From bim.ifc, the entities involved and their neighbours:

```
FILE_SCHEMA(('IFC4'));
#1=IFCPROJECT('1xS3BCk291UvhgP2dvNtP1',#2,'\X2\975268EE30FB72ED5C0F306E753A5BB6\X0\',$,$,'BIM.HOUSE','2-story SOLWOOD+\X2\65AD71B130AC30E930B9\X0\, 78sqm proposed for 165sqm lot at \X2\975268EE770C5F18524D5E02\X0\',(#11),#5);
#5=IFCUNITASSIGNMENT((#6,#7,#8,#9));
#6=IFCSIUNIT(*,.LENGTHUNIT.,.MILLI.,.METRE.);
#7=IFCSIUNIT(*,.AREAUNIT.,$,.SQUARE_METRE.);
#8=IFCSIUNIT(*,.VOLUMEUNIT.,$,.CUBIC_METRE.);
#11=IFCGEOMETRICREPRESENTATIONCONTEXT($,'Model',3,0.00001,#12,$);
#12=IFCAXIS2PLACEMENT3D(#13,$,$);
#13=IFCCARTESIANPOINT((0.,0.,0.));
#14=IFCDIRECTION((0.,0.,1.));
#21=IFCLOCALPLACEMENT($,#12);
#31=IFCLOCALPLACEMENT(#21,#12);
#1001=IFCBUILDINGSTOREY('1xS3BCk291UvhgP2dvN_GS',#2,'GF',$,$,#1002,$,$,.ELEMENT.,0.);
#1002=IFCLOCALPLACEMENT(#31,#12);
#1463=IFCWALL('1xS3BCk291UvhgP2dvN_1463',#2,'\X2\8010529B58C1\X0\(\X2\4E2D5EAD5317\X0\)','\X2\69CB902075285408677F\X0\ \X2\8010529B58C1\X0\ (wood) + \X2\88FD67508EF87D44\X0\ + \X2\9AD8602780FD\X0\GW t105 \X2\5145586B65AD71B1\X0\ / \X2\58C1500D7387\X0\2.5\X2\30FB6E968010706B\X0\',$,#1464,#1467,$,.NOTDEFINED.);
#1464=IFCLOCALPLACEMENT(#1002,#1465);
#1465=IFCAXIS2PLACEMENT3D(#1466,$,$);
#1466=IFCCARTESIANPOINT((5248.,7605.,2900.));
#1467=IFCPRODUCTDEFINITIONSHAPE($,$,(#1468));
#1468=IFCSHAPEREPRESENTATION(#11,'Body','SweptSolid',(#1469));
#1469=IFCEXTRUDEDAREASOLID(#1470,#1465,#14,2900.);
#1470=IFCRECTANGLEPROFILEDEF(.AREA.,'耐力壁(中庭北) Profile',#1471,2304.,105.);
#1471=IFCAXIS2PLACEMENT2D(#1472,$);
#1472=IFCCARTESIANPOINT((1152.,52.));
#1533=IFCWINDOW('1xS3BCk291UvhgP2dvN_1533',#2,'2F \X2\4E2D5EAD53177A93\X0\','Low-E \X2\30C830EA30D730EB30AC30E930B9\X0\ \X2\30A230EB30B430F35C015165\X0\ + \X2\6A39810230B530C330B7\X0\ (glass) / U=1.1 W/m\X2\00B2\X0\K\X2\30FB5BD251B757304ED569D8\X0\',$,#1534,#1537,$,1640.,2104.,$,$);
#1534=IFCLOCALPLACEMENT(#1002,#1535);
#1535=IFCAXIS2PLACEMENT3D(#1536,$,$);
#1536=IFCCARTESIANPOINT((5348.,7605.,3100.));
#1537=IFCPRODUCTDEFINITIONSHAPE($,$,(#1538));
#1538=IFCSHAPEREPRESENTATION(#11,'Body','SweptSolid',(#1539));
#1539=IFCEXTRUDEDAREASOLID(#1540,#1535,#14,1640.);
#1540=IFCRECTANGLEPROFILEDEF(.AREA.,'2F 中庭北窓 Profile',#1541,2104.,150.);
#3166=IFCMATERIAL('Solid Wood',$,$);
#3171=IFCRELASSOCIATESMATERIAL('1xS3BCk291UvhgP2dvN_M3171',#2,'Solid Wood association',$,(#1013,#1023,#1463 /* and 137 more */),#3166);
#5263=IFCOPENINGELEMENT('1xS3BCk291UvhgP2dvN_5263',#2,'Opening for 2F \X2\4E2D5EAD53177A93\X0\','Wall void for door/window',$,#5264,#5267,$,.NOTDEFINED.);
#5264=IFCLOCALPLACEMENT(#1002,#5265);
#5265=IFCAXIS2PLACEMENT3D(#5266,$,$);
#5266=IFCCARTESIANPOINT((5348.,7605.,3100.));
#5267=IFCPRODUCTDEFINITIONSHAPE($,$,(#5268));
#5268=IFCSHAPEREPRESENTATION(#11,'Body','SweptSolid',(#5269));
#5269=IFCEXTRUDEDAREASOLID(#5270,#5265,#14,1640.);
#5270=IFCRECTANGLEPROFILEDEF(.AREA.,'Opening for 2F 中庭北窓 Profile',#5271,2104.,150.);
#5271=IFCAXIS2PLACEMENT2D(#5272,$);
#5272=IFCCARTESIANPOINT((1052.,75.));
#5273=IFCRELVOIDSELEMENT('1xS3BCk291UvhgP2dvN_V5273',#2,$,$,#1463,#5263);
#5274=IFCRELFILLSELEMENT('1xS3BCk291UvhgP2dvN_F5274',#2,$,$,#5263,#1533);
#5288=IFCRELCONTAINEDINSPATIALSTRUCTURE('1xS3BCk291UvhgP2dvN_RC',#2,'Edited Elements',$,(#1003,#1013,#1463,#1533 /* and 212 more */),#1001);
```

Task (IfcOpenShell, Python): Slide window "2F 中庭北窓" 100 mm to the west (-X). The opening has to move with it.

```python
import ifcopenshell
import ifcopenshell.api.geometry
import ifcopenshell.util.placement
import ifcopenshell.util.unit

model = ifcopenshell.open("bim.ifc")
unit_scale = ifcopenshell.util.unit.calculate_unit_scale(model)

window = model.by_guid("1xS3BCk291UvhgP2dvN_1533")
opening = window.FillsVoids[0].RelatingOpeningElement
wall = opening.VoidsElements[0].RelatingBuildingElement

wall_matrix = ifcopenshell.util.placement.get_local_placement(wall.ObjectPlacement)
shift = wall_matrix[:3, 0] * -0.1 / unit_scale
before = ifcopenshell.util.placement.get_local_placement(window.ObjectPlacement)[:3, 3].copy()

# The window is not placed relative to its opening, so move both.
for product in (opening, window):
    matrix = ifcopenshell.util.placement.get_local_placement(product.ObjectPlacement)
    matrix[:3, 3] += shift
    ifcopenshell.api.geometry.edit_object_placement(model, product=product, matrix=matrix, is_si=False)

after = ifcopenshell.util.placement.get_local_placement(window.ObjectPlacement)[:3, 3]
print("window moved by", (after - before).round(3) + 0.0)

model.write("bim_v2.ifc")
```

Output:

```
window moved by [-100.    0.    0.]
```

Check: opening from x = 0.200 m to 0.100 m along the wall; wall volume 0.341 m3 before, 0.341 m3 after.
